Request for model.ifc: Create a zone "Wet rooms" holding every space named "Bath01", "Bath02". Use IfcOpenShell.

First a look at what the model holds.

```python
import ifcopenshell

model = ifcopenshell.open("model.ifc")
print(model.schema)
seen = {}
for space in model.by_type("IfcSpace"):
    seen[space.Name] = seen.get(space.Name, 0) + 1
for name, count in sorted(seen.items(), key=str):
    print(count, "x", name)
print("zones:", [z.Name for z in model.by_type("IfcZone")][:20])
```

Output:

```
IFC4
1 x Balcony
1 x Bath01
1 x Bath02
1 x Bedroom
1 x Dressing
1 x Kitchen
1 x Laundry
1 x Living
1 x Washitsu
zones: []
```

```python
import ifcopenshell
import ifcopenshell.api.group
import ifcopenshell.api.root

model = ifcopenshell.open("model.ifc")

names = {"Bath01", "Bath02"}
spaces = [s for s in model.by_type("IfcSpace") if s.Name in names]

zone = ifcopenshell.api.root.create_entity(model, ifc_class="IfcZone", name="Wet rooms")
ifcopenshell.api.group.assign_group(model, products=spaces, group=zone)
print(len(spaces), "spaces in", zone.Name)

model.write("model_updated.ifc")
```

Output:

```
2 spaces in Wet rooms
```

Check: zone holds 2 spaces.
